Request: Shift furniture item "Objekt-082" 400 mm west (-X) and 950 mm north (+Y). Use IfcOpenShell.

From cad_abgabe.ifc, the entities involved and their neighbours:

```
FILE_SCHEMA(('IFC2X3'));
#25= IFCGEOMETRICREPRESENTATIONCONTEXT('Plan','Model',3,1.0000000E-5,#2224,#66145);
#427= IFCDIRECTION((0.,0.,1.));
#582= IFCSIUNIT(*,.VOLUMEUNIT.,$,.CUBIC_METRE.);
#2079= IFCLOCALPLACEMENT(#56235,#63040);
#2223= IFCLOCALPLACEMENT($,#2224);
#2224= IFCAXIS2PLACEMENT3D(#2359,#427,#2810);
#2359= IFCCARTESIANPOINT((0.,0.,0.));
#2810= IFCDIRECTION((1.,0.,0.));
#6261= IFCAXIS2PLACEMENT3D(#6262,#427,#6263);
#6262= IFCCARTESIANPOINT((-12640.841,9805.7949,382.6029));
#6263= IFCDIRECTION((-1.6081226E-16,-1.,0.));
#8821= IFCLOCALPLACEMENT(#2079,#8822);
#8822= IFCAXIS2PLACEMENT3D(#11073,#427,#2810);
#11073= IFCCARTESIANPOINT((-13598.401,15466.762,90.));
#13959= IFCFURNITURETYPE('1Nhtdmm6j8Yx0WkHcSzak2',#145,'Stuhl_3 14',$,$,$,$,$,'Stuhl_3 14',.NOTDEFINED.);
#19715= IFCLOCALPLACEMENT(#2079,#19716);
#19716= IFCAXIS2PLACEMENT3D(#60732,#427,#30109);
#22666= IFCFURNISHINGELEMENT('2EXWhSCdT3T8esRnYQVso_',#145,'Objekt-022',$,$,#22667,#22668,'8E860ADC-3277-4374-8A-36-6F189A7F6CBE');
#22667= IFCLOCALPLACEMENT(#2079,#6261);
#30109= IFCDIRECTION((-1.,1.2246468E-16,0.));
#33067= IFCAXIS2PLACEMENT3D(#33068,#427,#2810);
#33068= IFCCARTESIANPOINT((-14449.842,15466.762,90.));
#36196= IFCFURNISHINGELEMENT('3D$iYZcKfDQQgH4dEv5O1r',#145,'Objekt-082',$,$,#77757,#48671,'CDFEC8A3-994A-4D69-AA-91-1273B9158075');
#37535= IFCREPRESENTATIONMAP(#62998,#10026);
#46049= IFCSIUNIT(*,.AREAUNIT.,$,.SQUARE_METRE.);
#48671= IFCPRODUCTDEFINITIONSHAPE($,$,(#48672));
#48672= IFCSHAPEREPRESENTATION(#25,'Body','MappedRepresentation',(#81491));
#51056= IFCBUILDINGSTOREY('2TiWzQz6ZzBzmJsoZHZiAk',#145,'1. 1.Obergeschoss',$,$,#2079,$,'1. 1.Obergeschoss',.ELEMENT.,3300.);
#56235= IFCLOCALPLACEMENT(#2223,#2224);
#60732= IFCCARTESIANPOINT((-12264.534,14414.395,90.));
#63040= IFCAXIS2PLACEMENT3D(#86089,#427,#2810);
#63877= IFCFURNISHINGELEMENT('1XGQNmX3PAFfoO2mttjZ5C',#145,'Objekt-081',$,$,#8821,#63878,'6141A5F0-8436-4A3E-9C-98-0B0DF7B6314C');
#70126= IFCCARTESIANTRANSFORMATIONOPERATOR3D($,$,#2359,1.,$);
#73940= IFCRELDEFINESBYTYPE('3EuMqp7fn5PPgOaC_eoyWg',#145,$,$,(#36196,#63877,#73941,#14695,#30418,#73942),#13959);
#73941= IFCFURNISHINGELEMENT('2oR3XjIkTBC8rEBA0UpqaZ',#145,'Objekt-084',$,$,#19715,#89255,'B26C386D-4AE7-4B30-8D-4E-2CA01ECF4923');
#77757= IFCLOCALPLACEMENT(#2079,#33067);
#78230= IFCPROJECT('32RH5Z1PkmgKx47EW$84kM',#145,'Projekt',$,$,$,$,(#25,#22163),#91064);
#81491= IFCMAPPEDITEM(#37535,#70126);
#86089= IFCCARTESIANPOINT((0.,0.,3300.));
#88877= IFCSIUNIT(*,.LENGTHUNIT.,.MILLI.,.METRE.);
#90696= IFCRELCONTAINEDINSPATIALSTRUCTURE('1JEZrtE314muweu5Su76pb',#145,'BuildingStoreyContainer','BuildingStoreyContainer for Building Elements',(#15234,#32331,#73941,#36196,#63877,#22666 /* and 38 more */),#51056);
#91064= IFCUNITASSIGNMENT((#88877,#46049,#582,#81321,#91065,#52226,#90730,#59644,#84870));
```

```python
import ifcopenshell
import ifcopenshell.api.geometry
import ifcopenshell.util.placement
import ifcopenshell.util.unit

model = ifcopenshell.open("cad_abgabe.ifc")
unit_scale = ifcopenshell.util.unit.calculate_unit_scale(model)

item = model.by_guid("3D$iYZcKfDQQgH4dEv5O1r")
matrix = ifcopenshell.util.placement.get_local_placement(item.ObjectPlacement)
matrix[0, 3] -= 0.4 / unit_scale
matrix[1, 3] += 0.95 / unit_scale
ifcopenshell.api.geometry.edit_object_placement(model, product=item, matrix=matrix, is_si=False)

print(ifcopenshell.util.placement.get_local_placement(item.ObjectPlacement).round(3) + 0.0)

model.write("cad_abgabe-out.ifc")
```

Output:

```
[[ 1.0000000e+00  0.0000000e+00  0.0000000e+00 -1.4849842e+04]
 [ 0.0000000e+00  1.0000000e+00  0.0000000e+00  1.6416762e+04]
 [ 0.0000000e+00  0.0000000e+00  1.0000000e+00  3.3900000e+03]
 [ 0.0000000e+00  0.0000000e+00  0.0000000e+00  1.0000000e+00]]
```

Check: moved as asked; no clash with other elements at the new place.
